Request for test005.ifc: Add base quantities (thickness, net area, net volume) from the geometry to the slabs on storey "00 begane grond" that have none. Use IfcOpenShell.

First a look at what the model holds.

```python
import ifcopenshell
import ifcopenshell.util.element
import ifcopenshell.util.unit

model = ifcopenshell.open("test005.ifc")
print(model.schema)
for unit_type in ("LENGTHUNIT", "AREAUNIT", "VOLUMEUNIT"):
    print(unit_type, ifcopenshell.util.unit.calculate_unit_scale(model, unit_type))
storey = next(s for s in model.by_type("IfcBuildingStorey") if s.Name == "00 begane grond")
slabs = [e for e in ifcopenshell.util.element.get_decomposition(storey) if e.is_a("IfcSlab")]
for e in sorted(slabs, key=lambda e: e.id()):
    print(e.id(), e.is_a(), e.Name, list(ifcopenshell.util.element.get_psets(e, qtos_only=True)), sep=" | ")
```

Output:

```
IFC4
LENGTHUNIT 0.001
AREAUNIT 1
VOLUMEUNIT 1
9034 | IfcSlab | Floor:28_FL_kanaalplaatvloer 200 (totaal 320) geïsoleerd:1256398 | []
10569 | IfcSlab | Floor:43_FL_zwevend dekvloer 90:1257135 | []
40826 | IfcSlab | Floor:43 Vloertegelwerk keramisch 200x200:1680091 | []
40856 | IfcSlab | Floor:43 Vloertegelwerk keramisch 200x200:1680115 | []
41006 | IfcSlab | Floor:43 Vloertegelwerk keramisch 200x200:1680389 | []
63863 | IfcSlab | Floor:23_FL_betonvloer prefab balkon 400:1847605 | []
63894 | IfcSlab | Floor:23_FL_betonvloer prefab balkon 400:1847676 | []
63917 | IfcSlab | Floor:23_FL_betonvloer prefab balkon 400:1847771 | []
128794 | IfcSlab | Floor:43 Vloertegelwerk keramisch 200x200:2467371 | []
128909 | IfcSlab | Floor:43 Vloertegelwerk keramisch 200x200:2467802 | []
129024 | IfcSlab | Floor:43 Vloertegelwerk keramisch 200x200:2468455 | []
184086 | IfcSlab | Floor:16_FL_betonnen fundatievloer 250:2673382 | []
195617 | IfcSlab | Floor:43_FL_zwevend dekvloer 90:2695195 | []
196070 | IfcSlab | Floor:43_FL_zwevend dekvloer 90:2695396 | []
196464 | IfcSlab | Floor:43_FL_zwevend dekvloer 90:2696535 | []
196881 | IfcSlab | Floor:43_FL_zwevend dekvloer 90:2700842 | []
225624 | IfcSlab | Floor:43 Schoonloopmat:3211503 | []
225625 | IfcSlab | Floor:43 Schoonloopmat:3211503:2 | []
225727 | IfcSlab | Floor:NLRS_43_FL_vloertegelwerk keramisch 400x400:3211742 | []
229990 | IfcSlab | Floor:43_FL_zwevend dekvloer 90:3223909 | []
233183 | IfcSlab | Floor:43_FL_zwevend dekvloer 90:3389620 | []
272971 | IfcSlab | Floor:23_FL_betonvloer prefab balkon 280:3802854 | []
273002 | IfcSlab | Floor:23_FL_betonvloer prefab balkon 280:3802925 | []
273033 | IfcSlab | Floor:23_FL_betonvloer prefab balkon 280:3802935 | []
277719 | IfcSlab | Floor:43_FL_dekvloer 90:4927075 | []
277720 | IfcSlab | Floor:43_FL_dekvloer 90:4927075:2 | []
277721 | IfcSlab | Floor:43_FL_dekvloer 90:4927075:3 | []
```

```python
import ifcopenshell
import ifcopenshell.api.pset
import ifcopenshell.geom
import ifcopenshell.util.element
import ifcopenshell.util.shape
import ifcopenshell.util.unit

model = ifcopenshell.open("test005.ifc")
unit_scale = ifcopenshell.util.unit.calculate_unit_scale(model)
area_scale = ifcopenshell.util.unit.calculate_unit_scale(model, "AREAUNIT")
volume_scale = ifcopenshell.util.unit.calculate_unit_scale(model, "VOLUMEUNIT")
settings = ifcopenshell.geom.settings()

storey = next(s for s in model.by_type("IfcBuildingStorey") if s.Name == "00 begane grond")
slabs = [e for e in ifcopenshell.util.element.get_decomposition(storey) if e.is_a("IfcSlab")]

for e in sorted(slabs, key=lambda e: e.id()):
    if ifcopenshell.util.element.get_psets(e, qtos_only=True, should_inherit=False):
        continue
    # Geometry comes back in metres, in the element's own axes.
    shape = ifcopenshell.geom.create_shape(settings, e)
    values = {
        "Width": ifcopenshell.util.shape.get_z(shape.geometry) / unit_scale,
        "NetArea": ifcopenshell.util.shape.get_footprint_area(shape.geometry) / area_scale,
        "NetVolume": ifcopenshell.util.shape.get_volume(shape.geometry) / volume_scale,
    }
    qto = ifcopenshell.api.pset.add_qto(model, product=e, name="Qto_SlabBaseQuantities")
    ifcopenshell.api.pset.edit_qto(model, qto=qto, properties=values)
    print(e.id(), {k: round(v, 3) for k, v in values.items()})

model.write("test005_v2.ifc")
```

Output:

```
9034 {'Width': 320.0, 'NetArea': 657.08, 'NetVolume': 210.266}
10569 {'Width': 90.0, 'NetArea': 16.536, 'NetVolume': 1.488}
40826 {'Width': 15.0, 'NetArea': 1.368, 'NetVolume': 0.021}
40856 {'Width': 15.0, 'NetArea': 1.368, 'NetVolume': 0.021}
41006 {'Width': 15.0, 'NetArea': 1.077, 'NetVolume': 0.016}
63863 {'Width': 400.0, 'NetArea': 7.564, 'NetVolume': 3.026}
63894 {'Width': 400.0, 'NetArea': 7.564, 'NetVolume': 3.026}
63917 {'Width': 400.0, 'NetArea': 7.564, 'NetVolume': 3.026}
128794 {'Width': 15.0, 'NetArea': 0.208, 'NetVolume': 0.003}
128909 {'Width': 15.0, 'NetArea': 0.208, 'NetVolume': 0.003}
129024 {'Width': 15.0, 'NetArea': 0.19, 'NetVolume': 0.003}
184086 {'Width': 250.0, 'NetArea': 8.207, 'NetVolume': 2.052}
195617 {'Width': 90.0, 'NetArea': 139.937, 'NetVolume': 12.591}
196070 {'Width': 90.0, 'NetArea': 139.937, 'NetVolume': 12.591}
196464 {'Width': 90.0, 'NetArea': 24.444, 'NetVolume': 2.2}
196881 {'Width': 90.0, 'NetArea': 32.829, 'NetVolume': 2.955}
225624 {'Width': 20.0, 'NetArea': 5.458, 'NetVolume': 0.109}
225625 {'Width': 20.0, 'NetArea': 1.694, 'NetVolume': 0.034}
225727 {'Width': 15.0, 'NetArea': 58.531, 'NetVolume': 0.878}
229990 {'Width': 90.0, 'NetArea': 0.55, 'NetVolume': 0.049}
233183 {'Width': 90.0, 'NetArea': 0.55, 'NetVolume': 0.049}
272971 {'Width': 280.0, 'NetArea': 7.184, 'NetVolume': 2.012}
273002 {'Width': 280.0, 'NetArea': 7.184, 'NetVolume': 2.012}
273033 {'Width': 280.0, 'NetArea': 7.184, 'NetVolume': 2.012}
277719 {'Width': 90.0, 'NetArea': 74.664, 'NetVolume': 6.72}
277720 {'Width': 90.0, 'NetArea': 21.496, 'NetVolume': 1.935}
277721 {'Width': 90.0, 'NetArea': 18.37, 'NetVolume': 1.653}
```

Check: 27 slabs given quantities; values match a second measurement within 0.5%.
